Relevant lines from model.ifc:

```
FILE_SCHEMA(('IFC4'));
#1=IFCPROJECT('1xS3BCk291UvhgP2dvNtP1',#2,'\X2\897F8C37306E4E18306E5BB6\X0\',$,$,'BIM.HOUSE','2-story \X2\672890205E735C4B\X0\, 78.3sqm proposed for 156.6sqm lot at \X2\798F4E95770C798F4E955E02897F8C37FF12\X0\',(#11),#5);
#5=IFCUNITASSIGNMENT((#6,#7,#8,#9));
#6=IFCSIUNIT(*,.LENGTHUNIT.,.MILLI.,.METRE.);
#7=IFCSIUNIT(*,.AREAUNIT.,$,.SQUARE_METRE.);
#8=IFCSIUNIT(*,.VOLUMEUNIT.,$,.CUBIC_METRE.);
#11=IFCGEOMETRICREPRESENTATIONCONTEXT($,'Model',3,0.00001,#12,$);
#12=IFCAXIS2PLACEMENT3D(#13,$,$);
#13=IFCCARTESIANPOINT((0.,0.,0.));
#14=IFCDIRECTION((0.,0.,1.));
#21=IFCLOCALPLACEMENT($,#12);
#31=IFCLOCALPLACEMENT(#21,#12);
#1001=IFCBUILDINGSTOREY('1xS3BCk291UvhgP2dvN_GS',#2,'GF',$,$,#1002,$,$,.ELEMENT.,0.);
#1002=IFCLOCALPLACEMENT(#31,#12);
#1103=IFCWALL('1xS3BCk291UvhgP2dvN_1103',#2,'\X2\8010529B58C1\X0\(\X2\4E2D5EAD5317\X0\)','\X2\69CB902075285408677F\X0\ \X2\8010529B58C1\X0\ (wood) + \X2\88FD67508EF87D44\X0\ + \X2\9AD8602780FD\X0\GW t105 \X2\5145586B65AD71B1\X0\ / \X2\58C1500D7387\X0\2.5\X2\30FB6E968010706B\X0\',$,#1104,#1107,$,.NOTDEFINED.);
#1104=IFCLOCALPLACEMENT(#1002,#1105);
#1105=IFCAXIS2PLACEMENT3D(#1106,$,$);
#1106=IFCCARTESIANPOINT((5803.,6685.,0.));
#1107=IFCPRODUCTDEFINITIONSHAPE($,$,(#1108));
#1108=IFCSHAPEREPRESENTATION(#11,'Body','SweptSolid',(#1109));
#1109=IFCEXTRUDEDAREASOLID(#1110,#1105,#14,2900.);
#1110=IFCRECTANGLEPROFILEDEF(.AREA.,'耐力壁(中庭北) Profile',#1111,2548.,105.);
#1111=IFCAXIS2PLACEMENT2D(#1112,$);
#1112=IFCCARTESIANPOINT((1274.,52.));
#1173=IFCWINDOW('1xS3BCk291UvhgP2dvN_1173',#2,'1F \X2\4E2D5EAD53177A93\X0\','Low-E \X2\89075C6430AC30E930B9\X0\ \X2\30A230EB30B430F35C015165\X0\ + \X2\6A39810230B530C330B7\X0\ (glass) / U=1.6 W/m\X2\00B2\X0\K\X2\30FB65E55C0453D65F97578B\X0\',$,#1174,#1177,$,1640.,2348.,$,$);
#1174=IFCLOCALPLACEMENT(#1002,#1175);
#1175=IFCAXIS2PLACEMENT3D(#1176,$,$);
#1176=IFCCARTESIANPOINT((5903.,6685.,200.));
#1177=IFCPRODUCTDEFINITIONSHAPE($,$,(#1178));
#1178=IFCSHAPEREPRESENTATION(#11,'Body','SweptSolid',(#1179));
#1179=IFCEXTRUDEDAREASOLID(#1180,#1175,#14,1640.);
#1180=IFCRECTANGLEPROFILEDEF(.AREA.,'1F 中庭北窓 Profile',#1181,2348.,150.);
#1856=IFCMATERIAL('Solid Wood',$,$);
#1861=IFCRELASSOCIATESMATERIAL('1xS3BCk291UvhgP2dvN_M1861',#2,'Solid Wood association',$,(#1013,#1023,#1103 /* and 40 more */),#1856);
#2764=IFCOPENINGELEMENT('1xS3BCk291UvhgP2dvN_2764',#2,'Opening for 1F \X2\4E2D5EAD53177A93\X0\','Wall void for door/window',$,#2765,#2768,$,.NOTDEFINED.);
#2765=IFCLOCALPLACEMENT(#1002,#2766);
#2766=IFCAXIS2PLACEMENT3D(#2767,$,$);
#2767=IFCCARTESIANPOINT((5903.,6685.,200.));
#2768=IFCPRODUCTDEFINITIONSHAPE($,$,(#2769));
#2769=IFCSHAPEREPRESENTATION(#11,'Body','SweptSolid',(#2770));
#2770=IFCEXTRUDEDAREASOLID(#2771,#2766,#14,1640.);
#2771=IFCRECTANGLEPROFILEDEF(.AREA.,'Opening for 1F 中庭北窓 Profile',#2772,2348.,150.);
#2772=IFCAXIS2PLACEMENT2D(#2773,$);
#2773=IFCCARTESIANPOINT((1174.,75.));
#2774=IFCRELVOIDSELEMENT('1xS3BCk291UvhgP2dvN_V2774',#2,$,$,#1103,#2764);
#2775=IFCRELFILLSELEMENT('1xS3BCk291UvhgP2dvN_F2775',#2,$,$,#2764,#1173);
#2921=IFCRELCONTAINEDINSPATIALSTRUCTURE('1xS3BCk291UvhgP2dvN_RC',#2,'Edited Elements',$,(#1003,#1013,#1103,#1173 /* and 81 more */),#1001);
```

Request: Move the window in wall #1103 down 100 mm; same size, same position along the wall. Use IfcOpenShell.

```python
import numpy as np
import ifcopenshell
import ifcopenshell.api.geometry
import ifcopenshell.util.placement
import ifcopenshell.util.unit

model = ifcopenshell.open("model.ifc")
unit_scale = ifcopenshell.util.unit.calculate_unit_scale(model)

window = model.by_guid("1xS3BCk291UvhgP2dvN_1173")
opening = window.FillsVoids[0].RelatingOpeningElement
dz = -0.1 / unit_scale

shift = np.array([0.0, 0.0, dz])
# The window is not placed relative to its opening, so move both.
for product in (opening, window):
    matrix = ifcopenshell.util.placement.get_local_placement(product.ObjectPlacement)
    matrix[:3, 3] += shift
    ifcopenshell.api.geometry.edit_object_placement(model, product=product, matrix=matrix, is_si=False)

print(f"moved by {dz * unit_scale:+.3f} m")

model.write("model_edited.ifc")
```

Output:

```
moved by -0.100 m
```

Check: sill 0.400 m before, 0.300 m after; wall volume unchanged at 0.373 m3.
